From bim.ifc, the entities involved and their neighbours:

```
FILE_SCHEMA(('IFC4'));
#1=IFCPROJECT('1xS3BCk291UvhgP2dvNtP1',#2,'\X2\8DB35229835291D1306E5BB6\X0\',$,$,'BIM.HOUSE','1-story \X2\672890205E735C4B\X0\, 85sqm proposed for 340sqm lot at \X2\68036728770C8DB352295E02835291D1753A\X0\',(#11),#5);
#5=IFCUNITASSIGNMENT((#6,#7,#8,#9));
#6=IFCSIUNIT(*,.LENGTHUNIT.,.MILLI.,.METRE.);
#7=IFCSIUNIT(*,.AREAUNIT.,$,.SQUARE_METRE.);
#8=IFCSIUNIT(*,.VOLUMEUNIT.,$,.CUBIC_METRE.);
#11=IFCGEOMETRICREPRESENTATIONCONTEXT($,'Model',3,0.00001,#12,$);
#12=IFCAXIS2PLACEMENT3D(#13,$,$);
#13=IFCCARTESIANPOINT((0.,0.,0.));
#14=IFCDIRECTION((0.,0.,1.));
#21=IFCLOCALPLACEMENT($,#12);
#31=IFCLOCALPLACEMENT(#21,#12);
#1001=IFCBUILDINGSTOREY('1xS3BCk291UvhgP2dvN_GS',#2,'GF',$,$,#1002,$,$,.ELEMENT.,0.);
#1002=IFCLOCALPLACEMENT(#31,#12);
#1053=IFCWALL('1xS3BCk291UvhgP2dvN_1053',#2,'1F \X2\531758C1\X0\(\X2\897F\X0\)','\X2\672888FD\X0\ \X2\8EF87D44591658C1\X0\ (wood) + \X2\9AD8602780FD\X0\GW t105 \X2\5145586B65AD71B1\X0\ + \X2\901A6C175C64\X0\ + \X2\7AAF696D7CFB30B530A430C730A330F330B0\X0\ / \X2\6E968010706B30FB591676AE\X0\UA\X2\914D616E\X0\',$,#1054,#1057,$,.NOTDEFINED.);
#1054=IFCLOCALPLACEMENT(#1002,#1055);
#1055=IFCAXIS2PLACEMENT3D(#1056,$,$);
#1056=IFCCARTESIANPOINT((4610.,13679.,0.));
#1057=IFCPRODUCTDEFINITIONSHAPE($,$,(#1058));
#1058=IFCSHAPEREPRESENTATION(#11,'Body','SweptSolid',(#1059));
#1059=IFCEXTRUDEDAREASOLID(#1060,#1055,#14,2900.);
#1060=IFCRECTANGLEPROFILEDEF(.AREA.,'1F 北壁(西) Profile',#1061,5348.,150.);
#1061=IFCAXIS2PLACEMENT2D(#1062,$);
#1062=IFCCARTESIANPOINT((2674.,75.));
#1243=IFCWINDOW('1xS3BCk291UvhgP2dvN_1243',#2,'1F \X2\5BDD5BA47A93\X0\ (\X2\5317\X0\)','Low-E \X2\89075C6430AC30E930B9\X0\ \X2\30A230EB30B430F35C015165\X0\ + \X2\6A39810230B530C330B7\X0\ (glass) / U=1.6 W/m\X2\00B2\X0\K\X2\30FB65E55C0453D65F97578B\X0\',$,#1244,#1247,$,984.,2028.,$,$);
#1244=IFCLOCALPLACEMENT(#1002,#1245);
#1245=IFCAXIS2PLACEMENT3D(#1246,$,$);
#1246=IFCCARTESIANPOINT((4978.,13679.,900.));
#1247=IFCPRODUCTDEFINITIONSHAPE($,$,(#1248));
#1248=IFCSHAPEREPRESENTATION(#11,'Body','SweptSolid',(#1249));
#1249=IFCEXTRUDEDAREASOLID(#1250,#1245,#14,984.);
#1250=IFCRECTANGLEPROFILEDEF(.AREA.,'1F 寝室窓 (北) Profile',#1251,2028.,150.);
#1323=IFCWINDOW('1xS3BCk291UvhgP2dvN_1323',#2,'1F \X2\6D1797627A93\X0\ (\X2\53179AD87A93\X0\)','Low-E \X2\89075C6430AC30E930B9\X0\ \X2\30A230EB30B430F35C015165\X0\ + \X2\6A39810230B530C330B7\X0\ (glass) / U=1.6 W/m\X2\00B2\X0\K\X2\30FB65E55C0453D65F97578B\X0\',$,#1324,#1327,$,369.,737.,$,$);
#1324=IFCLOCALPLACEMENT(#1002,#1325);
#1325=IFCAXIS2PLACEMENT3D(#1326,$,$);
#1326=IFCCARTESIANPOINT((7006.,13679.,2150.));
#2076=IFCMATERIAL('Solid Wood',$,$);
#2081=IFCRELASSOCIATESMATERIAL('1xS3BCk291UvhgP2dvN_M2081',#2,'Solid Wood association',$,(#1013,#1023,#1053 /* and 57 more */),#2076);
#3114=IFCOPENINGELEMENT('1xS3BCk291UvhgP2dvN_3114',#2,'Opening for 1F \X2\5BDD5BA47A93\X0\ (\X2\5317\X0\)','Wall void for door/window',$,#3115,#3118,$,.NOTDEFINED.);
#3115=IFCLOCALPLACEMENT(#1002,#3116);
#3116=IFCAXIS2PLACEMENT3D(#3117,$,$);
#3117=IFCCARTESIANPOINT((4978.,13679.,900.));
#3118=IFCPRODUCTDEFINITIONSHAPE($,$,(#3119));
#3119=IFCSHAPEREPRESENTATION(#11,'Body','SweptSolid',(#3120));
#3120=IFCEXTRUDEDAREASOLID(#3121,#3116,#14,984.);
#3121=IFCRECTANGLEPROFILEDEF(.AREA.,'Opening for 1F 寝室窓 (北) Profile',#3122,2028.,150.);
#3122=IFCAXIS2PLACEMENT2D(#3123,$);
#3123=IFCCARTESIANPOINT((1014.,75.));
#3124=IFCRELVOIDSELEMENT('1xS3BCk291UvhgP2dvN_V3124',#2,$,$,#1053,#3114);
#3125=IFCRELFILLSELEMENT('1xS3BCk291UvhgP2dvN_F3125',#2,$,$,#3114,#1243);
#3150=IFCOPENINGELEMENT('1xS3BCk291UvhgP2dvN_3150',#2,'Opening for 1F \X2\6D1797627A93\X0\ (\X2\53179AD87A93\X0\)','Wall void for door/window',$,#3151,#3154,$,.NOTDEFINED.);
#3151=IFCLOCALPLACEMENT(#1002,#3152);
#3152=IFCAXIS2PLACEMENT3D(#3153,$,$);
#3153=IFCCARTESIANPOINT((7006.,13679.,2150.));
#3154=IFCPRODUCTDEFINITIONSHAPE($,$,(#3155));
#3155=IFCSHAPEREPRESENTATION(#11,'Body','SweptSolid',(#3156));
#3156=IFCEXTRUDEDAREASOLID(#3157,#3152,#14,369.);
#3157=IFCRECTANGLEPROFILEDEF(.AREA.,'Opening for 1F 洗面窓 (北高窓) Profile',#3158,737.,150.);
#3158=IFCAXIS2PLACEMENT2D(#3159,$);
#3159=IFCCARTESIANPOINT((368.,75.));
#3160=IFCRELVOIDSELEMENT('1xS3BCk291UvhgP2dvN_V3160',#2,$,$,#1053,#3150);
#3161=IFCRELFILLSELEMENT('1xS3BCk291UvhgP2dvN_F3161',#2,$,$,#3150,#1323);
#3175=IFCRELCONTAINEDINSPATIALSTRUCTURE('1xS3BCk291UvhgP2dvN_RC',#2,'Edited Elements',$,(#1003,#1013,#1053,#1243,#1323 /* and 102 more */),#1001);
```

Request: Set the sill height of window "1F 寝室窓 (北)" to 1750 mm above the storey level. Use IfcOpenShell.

```python
import numpy as np
import ifcopenshell
import ifcopenshell.api.geometry
import ifcopenshell.geom
import ifcopenshell.util.element
import ifcopenshell.util.placement
import ifcopenshell.util.shape
import ifcopenshell.util.unit

model = ifcopenshell.open("bim.ifc")
unit_scale = ifcopenshell.util.unit.calculate_unit_scale(model)

window = model.by_guid("1xS3BCk291UvhgP2dvN_1243")
opening = window.FillsVoids[0].RelatingOpeningElement
storey = ifcopenshell.util.element.get_container(window, ifc_class="IfcBuildingStorey")
level = ifcopenshell.util.placement.get_local_placement(storey.ObjectPlacement)[2, 3]

# The opening's origin need not be at the sill, so measure its lowest point.
shape = ifcopenshell.geom.create_shape(ifcopenshell.geom.settings(), opening)
bottom = ifcopenshell.util.shape.get_shape_bottom_elevation(shape, shape.geometry) / unit_scale
dz = level + 1.75 / unit_scale - bottom

shift = np.array([0.0, 0.0, dz])
# The window is not placed relative to its opening, so move both.
for product in (opening, window):
    matrix = ifcopenshell.util.placement.get_local_placement(product.ObjectPlacement)
    matrix[:3, 3] += shift
    ifcopenshell.api.geometry.edit_object_placement(model, product=product, matrix=matrix, is_si=False)

print(f"moved by {dz * unit_scale:+.3f} m")

model.write("bim_updated.ifc")
```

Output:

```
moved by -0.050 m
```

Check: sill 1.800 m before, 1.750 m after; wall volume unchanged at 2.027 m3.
